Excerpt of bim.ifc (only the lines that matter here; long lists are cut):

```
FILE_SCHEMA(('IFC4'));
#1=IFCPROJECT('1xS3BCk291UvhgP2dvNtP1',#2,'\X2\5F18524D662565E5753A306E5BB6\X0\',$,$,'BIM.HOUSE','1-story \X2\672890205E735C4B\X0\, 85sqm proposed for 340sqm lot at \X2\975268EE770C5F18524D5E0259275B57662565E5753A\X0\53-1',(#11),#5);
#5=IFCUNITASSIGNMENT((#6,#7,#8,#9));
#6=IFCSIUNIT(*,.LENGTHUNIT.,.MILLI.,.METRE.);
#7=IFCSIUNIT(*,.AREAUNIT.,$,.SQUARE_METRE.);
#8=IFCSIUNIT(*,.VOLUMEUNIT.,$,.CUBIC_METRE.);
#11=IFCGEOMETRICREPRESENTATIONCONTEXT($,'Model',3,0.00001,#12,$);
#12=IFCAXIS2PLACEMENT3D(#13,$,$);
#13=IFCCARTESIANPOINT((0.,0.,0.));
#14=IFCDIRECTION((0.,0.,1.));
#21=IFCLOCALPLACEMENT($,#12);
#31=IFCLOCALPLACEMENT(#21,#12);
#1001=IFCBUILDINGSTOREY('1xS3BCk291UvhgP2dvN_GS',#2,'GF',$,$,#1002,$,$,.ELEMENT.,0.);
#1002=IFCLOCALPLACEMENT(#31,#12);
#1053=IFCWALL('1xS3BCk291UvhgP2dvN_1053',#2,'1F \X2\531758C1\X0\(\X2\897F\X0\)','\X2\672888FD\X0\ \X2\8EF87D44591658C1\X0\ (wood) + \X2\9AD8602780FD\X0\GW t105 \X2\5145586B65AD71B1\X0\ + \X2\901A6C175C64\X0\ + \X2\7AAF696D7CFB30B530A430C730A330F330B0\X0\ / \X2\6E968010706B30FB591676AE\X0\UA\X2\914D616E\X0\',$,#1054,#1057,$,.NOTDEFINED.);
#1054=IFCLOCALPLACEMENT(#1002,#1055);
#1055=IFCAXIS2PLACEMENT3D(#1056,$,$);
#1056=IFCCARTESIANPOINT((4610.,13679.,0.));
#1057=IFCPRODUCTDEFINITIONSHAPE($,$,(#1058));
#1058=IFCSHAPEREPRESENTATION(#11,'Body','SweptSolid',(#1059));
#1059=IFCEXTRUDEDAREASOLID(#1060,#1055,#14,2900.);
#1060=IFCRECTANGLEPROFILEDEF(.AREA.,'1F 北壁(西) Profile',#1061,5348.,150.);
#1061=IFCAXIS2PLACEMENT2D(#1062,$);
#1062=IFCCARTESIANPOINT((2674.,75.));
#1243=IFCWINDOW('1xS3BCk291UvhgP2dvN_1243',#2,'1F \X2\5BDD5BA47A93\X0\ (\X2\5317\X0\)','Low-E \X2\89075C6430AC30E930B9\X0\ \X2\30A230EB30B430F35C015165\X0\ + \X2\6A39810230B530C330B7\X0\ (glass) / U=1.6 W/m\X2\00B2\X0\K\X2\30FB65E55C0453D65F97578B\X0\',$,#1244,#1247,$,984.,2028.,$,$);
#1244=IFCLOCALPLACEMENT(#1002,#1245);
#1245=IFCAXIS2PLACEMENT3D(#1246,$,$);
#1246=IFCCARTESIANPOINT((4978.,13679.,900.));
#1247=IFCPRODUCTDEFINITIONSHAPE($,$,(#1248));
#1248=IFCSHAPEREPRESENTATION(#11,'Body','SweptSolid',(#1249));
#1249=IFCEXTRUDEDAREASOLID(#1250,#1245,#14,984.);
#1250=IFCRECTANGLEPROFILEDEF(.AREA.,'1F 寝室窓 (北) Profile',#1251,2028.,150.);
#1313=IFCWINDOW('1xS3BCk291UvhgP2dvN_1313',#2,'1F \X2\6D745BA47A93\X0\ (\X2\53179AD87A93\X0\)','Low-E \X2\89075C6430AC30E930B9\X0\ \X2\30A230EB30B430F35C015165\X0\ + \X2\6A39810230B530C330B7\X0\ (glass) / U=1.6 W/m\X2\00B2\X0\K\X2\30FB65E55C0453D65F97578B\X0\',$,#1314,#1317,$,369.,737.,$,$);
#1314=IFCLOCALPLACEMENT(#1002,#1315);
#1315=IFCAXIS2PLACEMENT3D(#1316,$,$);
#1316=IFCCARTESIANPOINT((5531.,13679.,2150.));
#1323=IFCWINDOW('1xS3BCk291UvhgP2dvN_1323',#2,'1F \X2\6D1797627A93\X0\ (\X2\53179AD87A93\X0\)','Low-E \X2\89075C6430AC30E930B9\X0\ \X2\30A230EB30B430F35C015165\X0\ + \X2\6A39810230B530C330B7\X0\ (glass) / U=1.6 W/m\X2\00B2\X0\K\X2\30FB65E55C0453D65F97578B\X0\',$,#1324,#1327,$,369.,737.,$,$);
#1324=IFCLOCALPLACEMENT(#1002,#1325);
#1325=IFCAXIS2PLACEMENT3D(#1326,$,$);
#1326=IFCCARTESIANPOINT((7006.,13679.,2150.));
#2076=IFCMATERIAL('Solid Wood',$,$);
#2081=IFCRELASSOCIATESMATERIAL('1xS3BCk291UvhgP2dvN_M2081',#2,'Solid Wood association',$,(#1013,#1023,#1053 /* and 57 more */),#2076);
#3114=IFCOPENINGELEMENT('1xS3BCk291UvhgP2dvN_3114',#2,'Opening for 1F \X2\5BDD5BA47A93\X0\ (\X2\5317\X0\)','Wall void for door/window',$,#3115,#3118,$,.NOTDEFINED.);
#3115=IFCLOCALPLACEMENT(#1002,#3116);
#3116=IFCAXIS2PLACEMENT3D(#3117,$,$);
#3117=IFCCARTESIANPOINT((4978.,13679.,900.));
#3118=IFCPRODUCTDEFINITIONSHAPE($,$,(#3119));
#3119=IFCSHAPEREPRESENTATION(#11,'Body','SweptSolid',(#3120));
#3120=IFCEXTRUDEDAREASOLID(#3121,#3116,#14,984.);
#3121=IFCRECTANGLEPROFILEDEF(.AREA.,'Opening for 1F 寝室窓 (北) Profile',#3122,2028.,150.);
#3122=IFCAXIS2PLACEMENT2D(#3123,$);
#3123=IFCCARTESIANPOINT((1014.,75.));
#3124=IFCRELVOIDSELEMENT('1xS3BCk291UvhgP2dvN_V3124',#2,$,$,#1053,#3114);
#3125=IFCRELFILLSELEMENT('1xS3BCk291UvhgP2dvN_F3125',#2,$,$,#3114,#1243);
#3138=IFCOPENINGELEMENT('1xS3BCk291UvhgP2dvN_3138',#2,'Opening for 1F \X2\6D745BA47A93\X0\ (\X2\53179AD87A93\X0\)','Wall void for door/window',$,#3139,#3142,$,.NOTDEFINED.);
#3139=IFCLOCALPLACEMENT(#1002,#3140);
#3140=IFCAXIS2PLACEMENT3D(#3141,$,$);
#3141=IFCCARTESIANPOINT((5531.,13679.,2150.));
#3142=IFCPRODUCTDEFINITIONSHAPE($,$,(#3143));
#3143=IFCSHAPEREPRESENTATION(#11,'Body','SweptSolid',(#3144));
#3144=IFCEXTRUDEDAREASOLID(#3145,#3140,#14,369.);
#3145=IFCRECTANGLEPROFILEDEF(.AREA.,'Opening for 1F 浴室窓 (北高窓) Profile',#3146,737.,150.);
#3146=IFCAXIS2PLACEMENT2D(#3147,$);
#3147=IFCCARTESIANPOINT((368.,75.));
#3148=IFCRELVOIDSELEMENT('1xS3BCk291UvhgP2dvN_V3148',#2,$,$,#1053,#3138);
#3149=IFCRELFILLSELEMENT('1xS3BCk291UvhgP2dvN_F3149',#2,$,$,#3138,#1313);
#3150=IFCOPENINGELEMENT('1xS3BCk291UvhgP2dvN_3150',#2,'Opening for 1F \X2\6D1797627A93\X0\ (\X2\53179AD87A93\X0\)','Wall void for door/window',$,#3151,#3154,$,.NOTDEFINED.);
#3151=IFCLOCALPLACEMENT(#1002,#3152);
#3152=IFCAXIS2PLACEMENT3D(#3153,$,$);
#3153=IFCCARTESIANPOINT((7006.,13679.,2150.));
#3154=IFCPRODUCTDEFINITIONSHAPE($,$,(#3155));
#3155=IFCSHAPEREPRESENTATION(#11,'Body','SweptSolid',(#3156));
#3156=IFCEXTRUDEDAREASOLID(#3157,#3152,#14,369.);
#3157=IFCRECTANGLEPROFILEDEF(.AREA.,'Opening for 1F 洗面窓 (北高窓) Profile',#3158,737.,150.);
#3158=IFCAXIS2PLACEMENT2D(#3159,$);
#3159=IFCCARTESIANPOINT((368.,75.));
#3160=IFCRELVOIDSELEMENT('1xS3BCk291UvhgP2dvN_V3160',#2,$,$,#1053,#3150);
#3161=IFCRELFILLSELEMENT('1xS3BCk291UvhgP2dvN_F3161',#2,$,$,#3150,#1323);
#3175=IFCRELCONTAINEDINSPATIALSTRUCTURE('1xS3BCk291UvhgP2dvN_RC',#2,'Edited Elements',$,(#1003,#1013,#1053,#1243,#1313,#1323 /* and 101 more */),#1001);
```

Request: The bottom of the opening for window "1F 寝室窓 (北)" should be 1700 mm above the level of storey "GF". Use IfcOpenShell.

```python
import numpy as np
import ifcopenshell
import ifcopenshell.api.geometry
import ifcopenshell.geom
import ifcopenshell.util.element
import ifcopenshell.util.placement
import ifcopenshell.util.shape
import ifcopenshell.util.unit

model = ifcopenshell.open("bim.ifc")
unit_scale = ifcopenshell.util.unit.calculate_unit_scale(model)

window = model.by_guid("1xS3BCk291UvhgP2dvN_1243")
opening = window.FillsVoids[0].RelatingOpeningElement
storey = ifcopenshell.util.element.get_container(window, ifc_class="IfcBuildingStorey")
level = ifcopenshell.util.placement.get_local_placement(storey.ObjectPlacement)[2, 3]

# The opening's origin need not be at the sill, so measure its lowest point.
shape = ifcopenshell.geom.create_shape(ifcopenshell.geom.settings(), opening)
bottom = ifcopenshell.util.shape.get_shape_bottom_elevation(shape, shape.geometry) / unit_scale
dz = level + 1.7 / unit_scale - bottom

shift = np.array([0.0, 0.0, dz])
# The window is not placed relative to its opening, so move both.
for product in (opening, window):
    matrix = ifcopenshell.util.placement.get_local_placement(product.ObjectPlacement)
    matrix[:3, 3] += shift
    ifcopenshell.api.geometry.edit_object_placement(model, product=product, matrix=matrix, is_si=False)

print(f"moved by {dz * unit_scale:+.3f} m")

model.write("bim_v2.ifc")
```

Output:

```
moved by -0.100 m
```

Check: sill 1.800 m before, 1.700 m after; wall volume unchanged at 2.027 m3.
